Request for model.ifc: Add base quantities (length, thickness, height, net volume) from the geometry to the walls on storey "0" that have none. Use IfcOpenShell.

First a look at what the model holds.

```python
import ifcopenshell
import ifcopenshell.util.element
import ifcopenshell.util.unit

model = ifcopenshell.open("model.ifc")
print(model.schema)
for unit_type in ("LENGTHUNIT", "AREAUNIT", "VOLUMEUNIT"):
    print(unit_type, ifcopenshell.util.unit.calculate_unit_scale(model, unit_type))
storey = next(s for s in model.by_type("IfcBuildingStorey") if s.Name == "0")
walls = [e for e in ifcopenshell.util.element.get_decomposition(storey) if e.is_a("IfcWall")]
for e in sorted(walls, key=lambda e: e.id()):
    print(e.id(), e.is_a(), e.Name, list(ifcopenshell.util.element.get_psets(e, qtos_only=True)), sep=" | ")
```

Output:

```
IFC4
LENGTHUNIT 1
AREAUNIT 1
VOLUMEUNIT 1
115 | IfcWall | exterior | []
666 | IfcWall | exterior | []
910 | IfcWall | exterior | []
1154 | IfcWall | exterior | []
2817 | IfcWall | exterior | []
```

```python
import ifcopenshell
import ifcopenshell.api.pset
import ifcopenshell.geom
import ifcopenshell.util.element
import ifcopenshell.util.shape
import ifcopenshell.util.unit

model = ifcopenshell.open("model.ifc")
unit_scale = ifcopenshell.util.unit.calculate_unit_scale(model)
volume_scale = ifcopenshell.util.unit.calculate_unit_scale(model, "VOLUMEUNIT")
settings = ifcopenshell.geom.settings()

storey = next(s for s in model.by_type("IfcBuildingStorey") if s.Name == "0")
walls = [e for e in ifcopenshell.util.element.get_decomposition(storey) if e.is_a("IfcWall")]

for e in sorted(walls, key=lambda e: e.id()):
    if ifcopenshell.util.element.get_psets(e, qtos_only=True, should_inherit=False):
        continue
    # Geometry comes back in metres, in the element's own axes.
    shape = ifcopenshell.geom.create_shape(settings, e)
    values = {
        "Length": ifcopenshell.util.shape.get_x(shape.geometry) / unit_scale,
        "Width": ifcopenshell.util.shape.get_y(shape.geometry) / unit_scale,
        "Height": ifcopenshell.util.shape.get_z(shape.geometry) / unit_scale,
        "NetVolume": ifcopenshell.util.shape.get_volume(shape.geometry) / volume_scale,
    }
    qto = ifcopenshell.api.pset.add_qto(model, product=e, name="Qto_WallBaseQuantities")
    ifcopenshell.api.pset.edit_qto(model, qto=qto, properties=values)
    print(e.id(), {k: round(v, 3) for k, v in values.items()})

model.write("model-out.ifc")
```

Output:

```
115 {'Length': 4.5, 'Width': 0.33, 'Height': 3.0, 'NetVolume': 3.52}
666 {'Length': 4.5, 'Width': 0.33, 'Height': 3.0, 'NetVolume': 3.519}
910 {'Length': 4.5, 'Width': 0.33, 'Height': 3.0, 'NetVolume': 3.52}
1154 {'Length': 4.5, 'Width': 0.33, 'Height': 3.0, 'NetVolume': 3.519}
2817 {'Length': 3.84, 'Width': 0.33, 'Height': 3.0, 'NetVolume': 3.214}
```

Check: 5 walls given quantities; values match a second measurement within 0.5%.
